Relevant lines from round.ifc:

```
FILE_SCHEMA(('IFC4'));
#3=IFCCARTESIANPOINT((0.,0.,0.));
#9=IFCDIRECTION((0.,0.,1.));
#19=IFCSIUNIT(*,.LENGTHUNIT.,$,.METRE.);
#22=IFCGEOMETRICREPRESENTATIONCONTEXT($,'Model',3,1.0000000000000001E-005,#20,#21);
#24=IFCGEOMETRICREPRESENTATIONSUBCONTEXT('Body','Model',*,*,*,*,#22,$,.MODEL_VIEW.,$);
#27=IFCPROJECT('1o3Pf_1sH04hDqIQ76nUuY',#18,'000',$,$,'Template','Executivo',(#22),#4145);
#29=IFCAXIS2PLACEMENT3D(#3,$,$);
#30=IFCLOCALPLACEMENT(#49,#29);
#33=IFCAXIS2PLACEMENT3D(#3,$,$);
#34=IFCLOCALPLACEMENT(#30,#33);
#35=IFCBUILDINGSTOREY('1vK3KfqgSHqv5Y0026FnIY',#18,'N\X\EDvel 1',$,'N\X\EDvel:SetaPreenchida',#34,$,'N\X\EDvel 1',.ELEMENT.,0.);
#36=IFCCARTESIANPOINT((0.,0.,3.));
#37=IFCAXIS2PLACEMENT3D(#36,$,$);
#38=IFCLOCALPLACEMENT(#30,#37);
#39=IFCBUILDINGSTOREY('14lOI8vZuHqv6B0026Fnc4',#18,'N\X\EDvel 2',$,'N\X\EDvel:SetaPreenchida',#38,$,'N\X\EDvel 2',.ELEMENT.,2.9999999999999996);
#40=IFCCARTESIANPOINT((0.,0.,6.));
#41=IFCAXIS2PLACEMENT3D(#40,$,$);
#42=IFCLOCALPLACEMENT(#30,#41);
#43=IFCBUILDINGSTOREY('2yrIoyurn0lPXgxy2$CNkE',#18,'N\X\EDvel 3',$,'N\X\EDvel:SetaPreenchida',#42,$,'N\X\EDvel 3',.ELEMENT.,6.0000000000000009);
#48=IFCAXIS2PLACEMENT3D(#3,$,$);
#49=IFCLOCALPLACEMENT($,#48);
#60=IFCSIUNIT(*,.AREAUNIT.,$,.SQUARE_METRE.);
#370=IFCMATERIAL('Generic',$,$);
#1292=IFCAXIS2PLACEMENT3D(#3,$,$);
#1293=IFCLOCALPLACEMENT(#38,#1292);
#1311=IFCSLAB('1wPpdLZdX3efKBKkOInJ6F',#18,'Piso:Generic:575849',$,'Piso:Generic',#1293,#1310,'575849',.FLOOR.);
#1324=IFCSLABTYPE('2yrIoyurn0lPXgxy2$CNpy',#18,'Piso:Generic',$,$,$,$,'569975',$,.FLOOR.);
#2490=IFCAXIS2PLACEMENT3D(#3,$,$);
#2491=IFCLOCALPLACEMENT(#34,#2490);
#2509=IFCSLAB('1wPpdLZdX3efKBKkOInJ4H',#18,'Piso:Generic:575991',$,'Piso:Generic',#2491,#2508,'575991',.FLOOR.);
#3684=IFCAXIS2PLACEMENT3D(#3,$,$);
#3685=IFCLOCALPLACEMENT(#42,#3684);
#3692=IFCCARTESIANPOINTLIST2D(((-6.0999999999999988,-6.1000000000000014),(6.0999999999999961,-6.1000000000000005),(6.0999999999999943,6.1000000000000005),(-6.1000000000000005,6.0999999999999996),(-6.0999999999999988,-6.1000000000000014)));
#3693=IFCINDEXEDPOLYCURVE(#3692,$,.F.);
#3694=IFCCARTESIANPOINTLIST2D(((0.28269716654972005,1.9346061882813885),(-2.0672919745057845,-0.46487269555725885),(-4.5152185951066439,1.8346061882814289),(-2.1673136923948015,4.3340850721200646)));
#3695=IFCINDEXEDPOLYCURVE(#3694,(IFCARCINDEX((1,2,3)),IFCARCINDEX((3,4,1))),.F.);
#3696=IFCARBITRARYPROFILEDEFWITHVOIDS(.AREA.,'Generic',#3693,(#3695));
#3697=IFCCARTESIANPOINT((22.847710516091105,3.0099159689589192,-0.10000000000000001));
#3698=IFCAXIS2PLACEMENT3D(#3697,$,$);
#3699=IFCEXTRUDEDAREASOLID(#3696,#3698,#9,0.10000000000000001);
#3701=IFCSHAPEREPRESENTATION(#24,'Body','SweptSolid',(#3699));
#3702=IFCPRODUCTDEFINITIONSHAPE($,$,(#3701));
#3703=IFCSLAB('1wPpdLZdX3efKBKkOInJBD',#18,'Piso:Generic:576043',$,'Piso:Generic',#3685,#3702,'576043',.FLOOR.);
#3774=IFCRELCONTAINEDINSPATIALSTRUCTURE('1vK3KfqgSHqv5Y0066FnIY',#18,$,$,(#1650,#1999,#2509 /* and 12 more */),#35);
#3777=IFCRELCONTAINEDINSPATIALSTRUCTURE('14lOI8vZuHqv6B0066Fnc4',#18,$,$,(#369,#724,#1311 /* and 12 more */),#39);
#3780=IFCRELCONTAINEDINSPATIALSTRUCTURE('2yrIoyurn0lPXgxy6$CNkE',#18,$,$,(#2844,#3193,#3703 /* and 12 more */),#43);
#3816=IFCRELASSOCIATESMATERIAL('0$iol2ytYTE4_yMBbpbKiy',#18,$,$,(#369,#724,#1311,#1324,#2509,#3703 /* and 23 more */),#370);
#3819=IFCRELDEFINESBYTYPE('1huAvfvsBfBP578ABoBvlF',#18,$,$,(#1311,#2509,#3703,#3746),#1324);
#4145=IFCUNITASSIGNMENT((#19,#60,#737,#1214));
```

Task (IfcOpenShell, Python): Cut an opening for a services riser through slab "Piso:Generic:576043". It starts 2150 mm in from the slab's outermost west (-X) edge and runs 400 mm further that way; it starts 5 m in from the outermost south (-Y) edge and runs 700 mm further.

```python
import numpy as np
import ifcopenshell
import ifcopenshell.api.feature
import ifcopenshell.api.geometry
import ifcopenshell.api.root
import ifcopenshell.geom
import ifcopenshell.util.placement
import ifcopenshell.util.representation
import ifcopenshell.util.shape
import ifcopenshell.util.unit

model = ifcopenshell.open("round.ifc")
unit_scale = ifcopenshell.util.unit.calculate_unit_scale(model)
settings = ifcopenshell.geom.settings()


def volume(element):
    """Net volume in cubic metres, openings subtracted."""
    shape = ifcopenshell.geom.create_shape(settings, element)
    return ifcopenshell.util.shape.get_volume(shape.geometry)


slab = model.by_guid("1wPpdLZdX3efKBKkOInJBD")
before = volume(slab)

# Extent in the slab's own axes, in metres. The edges named are its -X and -Y sides.
slab_shape = ifcopenshell.geom.create_shape(settings, slab)
vertices = ifcopenshell.util.shape.get_vertices(slab_shape.geometry)
x_min, y_min, bottom = vertices.min(axis=0)
top = vertices[:, 2].max()

opening = ifcopenshell.api.root.create_entity(model, ifc_class="IfcOpeningElement", name="Services riser opening", predefined_type="OPENING")
context = ifcopenshell.util.representation.get_context(model, "Model", "Body", "MODEL_VIEW")
width, depth = 0.4, 0.7
outline = [(0.0, 0.0), (width, 0.0), (width, depth), (0.0, depth), (0.0, 0.0)]
# Overshoot both faces by 50 mm so the cut is clean.
shape = ifcopenshell.api.geometry.add_slab_representation(
    model, context=context, depth=top - bottom + 0.1, polyline=outline
)
ifcopenshell.api.geometry.assign_representation(model, product=opening, representation=shape)

matrix = ifcopenshell.util.placement.get_local_placement(slab.ObjectPlacement)
matrix[:, 3] = matrix @ np.append(np.array([x_min + 2.15, y_min + 5, bottom - 0.05]) / unit_scale, 1.0)
ifcopenshell.api.geometry.edit_object_placement(model, product=opening, matrix=matrix, is_si=False)
ifcopenshell.api.feature.add_feature(model, feature=opening, element=slab)

after = volume(slab)

print(f"slab volume {before:.3f} -> {after:.3f} m3")

model.write("round-out.ifc")
```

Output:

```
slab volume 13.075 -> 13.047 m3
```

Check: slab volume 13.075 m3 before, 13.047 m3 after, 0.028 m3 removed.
